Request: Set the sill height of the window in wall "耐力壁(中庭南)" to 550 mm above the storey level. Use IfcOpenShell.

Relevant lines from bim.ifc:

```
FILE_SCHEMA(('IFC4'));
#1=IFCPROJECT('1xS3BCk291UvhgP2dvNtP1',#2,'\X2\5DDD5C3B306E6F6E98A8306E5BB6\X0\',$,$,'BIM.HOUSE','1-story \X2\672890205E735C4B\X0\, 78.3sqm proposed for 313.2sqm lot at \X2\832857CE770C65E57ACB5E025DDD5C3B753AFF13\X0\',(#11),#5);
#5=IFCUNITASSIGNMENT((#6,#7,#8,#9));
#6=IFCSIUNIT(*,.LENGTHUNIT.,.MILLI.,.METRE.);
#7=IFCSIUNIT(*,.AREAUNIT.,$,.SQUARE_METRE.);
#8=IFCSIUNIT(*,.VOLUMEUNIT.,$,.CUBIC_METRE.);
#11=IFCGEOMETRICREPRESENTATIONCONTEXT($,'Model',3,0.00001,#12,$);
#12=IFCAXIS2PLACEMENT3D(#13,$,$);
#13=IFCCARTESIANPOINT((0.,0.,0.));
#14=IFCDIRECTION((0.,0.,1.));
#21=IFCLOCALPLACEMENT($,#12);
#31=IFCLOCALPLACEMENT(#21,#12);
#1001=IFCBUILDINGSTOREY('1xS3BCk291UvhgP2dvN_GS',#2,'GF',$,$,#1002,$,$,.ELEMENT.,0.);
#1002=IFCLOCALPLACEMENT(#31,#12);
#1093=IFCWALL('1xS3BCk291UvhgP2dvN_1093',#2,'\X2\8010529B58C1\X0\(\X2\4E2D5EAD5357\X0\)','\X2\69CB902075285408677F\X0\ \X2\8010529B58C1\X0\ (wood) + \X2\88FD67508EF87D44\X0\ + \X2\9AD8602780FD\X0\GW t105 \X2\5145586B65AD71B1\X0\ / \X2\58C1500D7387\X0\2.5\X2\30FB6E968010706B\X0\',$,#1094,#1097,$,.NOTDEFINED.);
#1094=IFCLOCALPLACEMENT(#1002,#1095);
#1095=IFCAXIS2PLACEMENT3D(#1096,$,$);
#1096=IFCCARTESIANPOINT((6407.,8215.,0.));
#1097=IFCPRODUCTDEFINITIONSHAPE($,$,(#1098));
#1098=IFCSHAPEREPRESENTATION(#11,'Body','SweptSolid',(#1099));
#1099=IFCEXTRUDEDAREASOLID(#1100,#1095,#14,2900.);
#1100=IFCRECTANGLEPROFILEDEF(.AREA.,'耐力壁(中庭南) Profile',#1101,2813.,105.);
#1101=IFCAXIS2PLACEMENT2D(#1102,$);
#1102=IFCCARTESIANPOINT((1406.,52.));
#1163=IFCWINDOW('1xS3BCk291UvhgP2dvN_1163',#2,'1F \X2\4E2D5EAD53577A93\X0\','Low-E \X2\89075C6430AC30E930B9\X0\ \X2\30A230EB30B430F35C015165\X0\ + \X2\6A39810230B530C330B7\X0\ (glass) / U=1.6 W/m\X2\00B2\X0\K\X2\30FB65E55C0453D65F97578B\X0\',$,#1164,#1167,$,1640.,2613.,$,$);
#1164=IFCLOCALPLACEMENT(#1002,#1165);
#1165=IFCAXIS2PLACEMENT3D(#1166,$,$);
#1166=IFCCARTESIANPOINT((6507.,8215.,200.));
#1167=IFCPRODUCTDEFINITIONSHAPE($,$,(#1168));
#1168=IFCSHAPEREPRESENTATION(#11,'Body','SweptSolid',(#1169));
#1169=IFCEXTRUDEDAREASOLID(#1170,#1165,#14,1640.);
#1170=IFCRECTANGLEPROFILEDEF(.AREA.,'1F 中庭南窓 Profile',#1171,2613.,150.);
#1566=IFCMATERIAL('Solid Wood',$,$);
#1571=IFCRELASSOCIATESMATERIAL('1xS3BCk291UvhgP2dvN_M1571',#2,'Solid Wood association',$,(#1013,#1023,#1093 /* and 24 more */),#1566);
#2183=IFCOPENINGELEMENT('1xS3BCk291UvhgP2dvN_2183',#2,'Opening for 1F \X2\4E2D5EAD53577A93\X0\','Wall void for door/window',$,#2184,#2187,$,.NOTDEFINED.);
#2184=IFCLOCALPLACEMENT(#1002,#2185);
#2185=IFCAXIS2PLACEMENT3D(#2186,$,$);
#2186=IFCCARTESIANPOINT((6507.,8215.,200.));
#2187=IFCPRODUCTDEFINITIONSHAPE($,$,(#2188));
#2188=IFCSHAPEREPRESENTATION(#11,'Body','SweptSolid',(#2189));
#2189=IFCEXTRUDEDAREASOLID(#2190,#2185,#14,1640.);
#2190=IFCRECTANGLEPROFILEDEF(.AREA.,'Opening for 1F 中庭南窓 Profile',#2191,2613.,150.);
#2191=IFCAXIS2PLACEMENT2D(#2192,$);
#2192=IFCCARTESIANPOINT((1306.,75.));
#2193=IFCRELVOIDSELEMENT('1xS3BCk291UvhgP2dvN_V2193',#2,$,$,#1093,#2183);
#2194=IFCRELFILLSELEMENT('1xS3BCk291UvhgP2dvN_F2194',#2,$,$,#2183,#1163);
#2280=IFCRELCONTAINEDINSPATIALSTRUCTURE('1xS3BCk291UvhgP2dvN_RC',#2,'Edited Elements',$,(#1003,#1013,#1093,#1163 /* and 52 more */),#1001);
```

```python
import numpy as np
import ifcopenshell
import ifcopenshell.api.geometry
import ifcopenshell.geom
import ifcopenshell.util.element
import ifcopenshell.util.placement
import ifcopenshell.util.shape
import ifcopenshell.util.unit

model = ifcopenshell.open("bim.ifc")
unit_scale = ifcopenshell.util.unit.calculate_unit_scale(model)

window = model.by_guid("1xS3BCk291UvhgP2dvN_1163")
opening = window.FillsVoids[0].RelatingOpeningElement
storey = ifcopenshell.util.element.get_container(window, ifc_class="IfcBuildingStorey")
level = ifcopenshell.util.placement.get_local_placement(storey.ObjectPlacement)[2, 3]

# The opening's origin need not be at the sill, so measure its lowest point.
shape = ifcopenshell.geom.create_shape(ifcopenshell.geom.settings(), opening)
bottom = ifcopenshell.util.shape.get_shape_bottom_elevation(shape, shape.geometry) / unit_scale
dz = level + 0.55 / unit_scale - bottom

shift = np.array([0.0, 0.0, dz])
# The window is not placed relative to its opening, so move both.
for product in (opening, window):
    matrix = ifcopenshell.util.placement.get_local_placement(product.ObjectPlacement)
    matrix[:3, 3] += shift
    ifcopenshell.api.geometry.edit_object_placement(model, product=product, matrix=matrix, is_si=False)

print(f"moved by {dz * unit_scale:+.3f} m")

model.write("bim_v2.ifc")
```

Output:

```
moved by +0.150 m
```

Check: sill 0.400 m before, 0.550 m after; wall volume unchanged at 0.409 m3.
